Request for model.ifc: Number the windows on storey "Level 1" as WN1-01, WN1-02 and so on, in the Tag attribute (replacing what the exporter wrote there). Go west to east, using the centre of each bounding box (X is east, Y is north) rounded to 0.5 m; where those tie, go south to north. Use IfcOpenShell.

First a look at what the model holds.

```python
import ifcopenshell
import ifcopenshell.util.element
import ifcopenshell.util.placement

model = ifcopenshell.open("model.ifc")
print(model.schema)
storey = next(s for s in model.by_type("IfcBuildingStorey") if s.Name == "Level 1")
windows = [e for e in ifcopenshell.util.element.get_decomposition(storey) if e.is_a("IfcWindow")]
for e in sorted(windows, key=lambda e: e.id()):
    origin = ifcopenshell.util.placement.get_local_placement(e.ObjectPlacement)[:3, 3]
    print(e.id(), e.Tag, e.Name, origin.round(2) + 0.0, sep=" | ")
```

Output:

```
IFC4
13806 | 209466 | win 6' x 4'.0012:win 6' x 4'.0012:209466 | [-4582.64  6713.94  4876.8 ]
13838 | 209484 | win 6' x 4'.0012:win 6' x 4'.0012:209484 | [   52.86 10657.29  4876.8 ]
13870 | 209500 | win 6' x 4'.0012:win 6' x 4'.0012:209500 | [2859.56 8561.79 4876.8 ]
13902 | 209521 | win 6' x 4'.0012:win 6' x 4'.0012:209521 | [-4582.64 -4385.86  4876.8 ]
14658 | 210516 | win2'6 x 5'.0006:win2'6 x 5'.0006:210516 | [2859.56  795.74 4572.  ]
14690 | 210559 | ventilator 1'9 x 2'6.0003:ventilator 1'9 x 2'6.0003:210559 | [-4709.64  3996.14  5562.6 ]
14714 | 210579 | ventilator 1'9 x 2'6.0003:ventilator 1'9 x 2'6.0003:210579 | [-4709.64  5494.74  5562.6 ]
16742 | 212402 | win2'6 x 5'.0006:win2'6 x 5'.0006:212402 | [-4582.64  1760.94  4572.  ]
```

```python
import ifcopenshell
import ifcopenshell.geom
import ifcopenshell.util.element
import ifcopenshell.util.shape

model = ifcopenshell.open("model.ifc")
settings = ifcopenshell.geom.settings()
settings.set("use-world-coords", True)


def centre(element):
    shape = ifcopenshell.geom.create_shape(settings, element)
    return ifcopenshell.util.shape.get_bbox_centroid(shape.geometry)


storey = next(s for s in model.by_type("IfcBuildingStorey") if s.Name == "Level 1")
windows = [e for e in ifcopenshell.util.element.get_decomposition(storey) if e.is_a("IfcWindow")]

# Insertion points can sit at a corner or the storey origin, so sort by the geometry (in metres).
centres = {e: centre(e) for e in windows}
windows.sort(key=lambda e: (round(centres[e][0] / 0.5), centres[e][1]))

for i, e in enumerate(windows, start=1):
    number = f"WN1-{i:02d}"
    e.Tag = number
    print(e.id(), number)

model.write("model_updated.ifc")
```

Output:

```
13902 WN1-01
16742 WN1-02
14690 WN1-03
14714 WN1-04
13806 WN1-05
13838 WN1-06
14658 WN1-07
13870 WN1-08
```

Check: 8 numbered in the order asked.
